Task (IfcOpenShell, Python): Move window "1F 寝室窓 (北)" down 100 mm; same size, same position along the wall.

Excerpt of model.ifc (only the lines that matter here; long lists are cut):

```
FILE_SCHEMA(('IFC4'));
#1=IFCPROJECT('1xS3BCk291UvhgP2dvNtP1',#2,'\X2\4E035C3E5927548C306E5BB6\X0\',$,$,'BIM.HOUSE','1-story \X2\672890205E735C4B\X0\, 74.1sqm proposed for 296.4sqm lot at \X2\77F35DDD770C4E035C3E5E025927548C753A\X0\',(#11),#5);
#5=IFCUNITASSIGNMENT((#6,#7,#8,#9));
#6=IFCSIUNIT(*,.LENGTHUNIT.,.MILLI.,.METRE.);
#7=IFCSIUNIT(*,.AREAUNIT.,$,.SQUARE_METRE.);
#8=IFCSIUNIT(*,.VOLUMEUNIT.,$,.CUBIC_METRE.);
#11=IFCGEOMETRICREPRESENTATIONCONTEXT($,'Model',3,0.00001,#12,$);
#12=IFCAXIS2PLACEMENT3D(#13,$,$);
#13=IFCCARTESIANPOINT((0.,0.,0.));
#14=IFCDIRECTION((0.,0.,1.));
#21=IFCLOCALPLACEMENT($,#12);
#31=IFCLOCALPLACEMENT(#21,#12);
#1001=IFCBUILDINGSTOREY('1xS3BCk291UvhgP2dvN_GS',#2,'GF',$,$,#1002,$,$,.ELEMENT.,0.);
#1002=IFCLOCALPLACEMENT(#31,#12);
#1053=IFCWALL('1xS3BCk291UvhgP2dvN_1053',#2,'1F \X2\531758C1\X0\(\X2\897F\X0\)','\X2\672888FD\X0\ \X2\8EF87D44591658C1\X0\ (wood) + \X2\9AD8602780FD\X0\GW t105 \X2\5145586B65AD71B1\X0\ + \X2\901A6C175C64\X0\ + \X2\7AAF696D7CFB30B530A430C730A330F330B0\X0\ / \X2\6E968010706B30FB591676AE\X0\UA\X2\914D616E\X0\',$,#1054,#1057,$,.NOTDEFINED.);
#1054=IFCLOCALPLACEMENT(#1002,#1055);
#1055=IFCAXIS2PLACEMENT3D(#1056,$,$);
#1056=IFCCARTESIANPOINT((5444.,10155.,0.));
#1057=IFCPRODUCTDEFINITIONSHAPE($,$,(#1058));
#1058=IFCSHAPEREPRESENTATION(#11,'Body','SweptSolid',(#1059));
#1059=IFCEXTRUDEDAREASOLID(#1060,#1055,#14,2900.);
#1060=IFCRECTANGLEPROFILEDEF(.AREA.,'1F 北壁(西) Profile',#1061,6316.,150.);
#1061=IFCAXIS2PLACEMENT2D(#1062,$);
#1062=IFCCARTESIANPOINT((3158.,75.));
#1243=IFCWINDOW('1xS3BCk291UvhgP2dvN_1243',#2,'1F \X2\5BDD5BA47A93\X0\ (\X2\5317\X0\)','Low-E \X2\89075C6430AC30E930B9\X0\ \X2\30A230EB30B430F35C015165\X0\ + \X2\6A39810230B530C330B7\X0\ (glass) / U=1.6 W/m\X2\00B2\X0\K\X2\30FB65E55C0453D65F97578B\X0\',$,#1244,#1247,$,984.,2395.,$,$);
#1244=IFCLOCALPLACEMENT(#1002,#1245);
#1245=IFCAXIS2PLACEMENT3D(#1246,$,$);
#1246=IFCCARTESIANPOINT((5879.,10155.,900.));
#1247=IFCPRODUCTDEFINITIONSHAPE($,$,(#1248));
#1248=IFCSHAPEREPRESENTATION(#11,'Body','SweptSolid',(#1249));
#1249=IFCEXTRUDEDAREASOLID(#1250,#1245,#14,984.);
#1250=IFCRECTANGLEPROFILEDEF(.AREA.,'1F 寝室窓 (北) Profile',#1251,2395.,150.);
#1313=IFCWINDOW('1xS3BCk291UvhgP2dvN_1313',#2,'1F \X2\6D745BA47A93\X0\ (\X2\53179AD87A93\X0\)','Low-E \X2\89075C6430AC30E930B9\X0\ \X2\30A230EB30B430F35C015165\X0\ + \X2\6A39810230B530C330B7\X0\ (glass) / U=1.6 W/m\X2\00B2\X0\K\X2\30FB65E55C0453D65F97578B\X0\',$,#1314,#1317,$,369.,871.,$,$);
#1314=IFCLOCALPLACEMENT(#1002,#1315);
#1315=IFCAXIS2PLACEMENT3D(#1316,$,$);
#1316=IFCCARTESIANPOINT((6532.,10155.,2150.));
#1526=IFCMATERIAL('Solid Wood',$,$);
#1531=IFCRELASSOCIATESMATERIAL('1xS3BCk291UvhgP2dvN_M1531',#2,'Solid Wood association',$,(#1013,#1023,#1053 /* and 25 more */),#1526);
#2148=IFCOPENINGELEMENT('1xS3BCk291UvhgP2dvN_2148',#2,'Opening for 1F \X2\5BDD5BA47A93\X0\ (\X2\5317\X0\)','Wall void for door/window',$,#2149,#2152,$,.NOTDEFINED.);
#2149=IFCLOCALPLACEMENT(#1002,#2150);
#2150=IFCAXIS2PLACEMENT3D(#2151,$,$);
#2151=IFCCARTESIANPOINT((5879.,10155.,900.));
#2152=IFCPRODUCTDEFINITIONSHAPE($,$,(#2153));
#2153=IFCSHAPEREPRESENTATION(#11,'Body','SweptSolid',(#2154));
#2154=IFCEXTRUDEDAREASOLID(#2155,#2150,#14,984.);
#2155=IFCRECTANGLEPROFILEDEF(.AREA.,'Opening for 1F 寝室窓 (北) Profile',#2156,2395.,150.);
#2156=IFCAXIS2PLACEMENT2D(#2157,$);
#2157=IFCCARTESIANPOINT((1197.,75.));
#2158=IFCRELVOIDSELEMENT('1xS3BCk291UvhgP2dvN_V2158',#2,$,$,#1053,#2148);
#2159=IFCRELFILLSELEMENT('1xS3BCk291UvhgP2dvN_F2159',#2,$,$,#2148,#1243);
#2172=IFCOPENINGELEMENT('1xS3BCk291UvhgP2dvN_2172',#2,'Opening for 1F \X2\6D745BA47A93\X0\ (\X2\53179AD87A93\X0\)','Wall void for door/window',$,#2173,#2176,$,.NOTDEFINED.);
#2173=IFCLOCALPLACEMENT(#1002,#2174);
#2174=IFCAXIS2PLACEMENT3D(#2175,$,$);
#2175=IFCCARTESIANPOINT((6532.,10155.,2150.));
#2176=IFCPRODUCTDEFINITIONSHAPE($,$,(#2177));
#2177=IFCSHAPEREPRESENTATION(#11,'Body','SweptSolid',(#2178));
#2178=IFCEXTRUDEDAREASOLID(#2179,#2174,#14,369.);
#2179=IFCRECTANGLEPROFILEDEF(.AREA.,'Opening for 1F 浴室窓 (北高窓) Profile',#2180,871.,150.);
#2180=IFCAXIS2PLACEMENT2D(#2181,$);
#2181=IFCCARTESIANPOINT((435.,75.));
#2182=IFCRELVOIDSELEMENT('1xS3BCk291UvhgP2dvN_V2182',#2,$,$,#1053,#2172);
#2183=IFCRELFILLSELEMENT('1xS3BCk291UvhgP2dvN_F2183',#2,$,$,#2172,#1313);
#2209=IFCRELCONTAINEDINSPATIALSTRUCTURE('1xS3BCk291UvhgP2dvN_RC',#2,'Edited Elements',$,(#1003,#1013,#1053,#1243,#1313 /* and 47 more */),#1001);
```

```python
import numpy as np
import ifcopenshell
import ifcopenshell.api.geometry
import ifcopenshell.util.placement
import ifcopenshell.util.unit

model = ifcopenshell.open("model.ifc")
unit_scale = ifcopenshell.util.unit.calculate_unit_scale(model)

window = model.by_guid("1xS3BCk291UvhgP2dvN_1243")
opening = window.FillsVoids[0].RelatingOpeningElement
dz = -100.0

shift = np.array([0.0, 0.0, dz])
# The window is not placed relative to its opening, so move both.
for product in (opening, window):
    matrix = ifcopenshell.util.placement.get_local_placement(product.ObjectPlacement)
    matrix[:3, 3] += shift
    ifcopenshell.api.geometry.edit_object_placement(model, product=product, matrix=matrix, is_si=False)

print(f"moved by {dz * unit_scale:+.3f} m")

model.write("model_rev.ifc")
```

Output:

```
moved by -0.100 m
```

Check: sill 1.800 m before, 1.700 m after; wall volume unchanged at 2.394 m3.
